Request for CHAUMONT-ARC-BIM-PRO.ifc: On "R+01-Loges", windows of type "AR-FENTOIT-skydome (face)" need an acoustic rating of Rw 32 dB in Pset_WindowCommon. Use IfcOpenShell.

First a look at what the model holds.

```python
import ifcopenshell
import ifcopenshell.util.element

model = ifcopenshell.open("CHAUMONT-ARC-BIM-PRO.ifc")
print(model.schema)
storey = next(s for s in model.by_type("IfcBuildingStorey") if s.Name == "R+01-Loges")
windows = [e for e in ifcopenshell.util.element.get_decomposition(storey) if e.is_a("IfcWindow")]
seen = {}
for e in windows:
    element_type = ifcopenshell.util.element.get_type(e)
    key = (element_type.Name if element_type != e and element_type else None, ifcopenshell.util.element.get_pset(e, "Pset_WindowCommon", "AcousticRating"))
    seen[key] = seen.get(key, 0) + 1
for (name, value), count in sorted(seen.items(), key=str):
    print(count, "x", name, "|", value)
```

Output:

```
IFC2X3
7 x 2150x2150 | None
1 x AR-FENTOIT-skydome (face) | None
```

```python
import ifcopenshell
import ifcopenshell.api.pset
import ifcopenshell.util.element

model = ifcopenshell.open("CHAUMONT-ARC-BIM-PRO.ifc")

storey = next(s for s in model.by_type("IfcBuildingStorey") if s.Name == "R+01-Loges")
windows = [e for e in ifcopenshell.util.element.get_decomposition(storey) if e.is_a("IfcWindow")]

count = 0
for e in windows:
    element_type = ifcopenshell.util.element.get_type(e)
    if element_type in (None, e) or element_type.Name != "AR-FENTOIT-skydome (face)":
        continue
    # add_pset returns the element's existing set when there is one.
    pset = ifcopenshell.api.pset.add_pset(model, product=e, name="Pset_WindowCommon")
    ifcopenshell.api.pset.edit_pset(model, pset=pset, properties={"AcousticRating": "Rw 32 dB"})
    count += 1

print(count, "windows updated")

model.write("CHAUMONT-ARC-BIM-PRO-out.ifc")
```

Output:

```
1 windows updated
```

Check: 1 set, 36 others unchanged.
